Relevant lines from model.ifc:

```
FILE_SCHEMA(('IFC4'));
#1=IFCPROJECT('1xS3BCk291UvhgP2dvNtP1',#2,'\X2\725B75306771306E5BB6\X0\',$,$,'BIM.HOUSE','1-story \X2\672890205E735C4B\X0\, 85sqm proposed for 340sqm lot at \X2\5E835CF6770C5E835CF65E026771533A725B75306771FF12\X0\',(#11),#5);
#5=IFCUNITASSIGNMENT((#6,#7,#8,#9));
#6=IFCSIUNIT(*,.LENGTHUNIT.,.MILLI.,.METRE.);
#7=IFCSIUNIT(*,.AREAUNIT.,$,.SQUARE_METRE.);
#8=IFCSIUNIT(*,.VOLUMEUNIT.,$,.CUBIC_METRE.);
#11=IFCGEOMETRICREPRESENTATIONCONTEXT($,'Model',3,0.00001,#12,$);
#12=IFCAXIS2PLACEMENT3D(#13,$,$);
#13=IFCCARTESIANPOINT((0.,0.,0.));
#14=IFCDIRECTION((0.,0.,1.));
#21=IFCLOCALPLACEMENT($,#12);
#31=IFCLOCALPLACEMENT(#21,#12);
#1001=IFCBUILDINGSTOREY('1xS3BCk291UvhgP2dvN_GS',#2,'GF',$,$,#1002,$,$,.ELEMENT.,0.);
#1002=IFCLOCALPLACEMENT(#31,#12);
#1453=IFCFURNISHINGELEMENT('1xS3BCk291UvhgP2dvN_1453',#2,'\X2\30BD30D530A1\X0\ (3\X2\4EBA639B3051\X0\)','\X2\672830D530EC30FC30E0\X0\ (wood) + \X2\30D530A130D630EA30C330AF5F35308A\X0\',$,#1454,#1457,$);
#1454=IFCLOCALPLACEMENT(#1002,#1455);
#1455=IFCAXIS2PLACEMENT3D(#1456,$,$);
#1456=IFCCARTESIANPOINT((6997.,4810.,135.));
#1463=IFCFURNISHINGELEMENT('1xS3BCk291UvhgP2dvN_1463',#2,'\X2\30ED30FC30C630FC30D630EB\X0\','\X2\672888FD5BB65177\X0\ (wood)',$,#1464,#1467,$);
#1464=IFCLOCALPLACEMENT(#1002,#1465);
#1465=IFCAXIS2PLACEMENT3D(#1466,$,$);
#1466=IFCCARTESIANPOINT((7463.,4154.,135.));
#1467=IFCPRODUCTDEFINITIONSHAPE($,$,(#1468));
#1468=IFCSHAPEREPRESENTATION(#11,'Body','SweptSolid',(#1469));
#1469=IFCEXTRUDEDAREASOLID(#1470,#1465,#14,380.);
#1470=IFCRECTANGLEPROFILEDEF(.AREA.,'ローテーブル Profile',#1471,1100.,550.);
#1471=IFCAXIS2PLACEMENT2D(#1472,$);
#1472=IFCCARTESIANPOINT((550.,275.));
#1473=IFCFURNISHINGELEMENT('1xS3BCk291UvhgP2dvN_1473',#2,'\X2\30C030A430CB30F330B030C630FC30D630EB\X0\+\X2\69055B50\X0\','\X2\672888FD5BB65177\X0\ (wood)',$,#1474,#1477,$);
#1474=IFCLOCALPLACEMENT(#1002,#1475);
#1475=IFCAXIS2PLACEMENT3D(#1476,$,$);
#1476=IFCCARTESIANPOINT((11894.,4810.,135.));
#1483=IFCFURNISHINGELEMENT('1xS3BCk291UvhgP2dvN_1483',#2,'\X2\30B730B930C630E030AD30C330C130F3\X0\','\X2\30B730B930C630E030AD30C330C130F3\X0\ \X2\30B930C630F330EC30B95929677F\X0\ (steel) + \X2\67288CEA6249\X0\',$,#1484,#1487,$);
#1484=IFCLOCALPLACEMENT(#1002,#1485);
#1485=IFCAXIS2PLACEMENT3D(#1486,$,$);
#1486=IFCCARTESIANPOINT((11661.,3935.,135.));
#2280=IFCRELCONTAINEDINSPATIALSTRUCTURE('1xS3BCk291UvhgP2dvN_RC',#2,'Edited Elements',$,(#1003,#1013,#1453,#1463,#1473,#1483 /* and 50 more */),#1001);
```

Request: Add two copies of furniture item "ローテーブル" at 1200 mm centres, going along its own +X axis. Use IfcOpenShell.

```python
import ifcopenshell
import ifcopenshell.api.geometry
import ifcopenshell.api.root
import ifcopenshell.util.element
import ifcopenshell.util.placement

model = ifcopenshell.open("model.ifc")


def reuse_history(source, copy):
    """copy_class also copies each property set's owner history, people and application; keep the originals."""
    for rel in copy.IsDefinedBy:
        if rel.is_a("IfcRelDefinesByProperties") and (history := rel.RelatingPropertyDefinition.OwnerHistory):
            rel.RelatingPropertyDefinition.OwnerHistory = source.OwnerHistory
            ifcopenshell.util.element.remove_deep2(model, history)


source = model.by_guid("1xS3BCk291UvhgP2dvN_1463")
base = ifcopenshell.util.placement.get_local_placement(source.ObjectPlacement)
step = base[:3, 0] * 1200.0

for i in range(1, 3):
    copy = ifcopenshell.api.root.copy_class(model, product=source)
    copy.Representation = ifcopenshell.util.element.copy_deep(
        model, source.Representation, exclude=["IfcGeometricRepresentationContext", "IfcRepresentationMap"]
    )
    reuse_history(source, copy)
    matrix = base.copy()
    matrix[:3, 3] += i * step
    print("added at", matrix[:3, 3].round(3) + 0.0)
    ifcopenshell.api.geometry.edit_object_placement(model, product=copy, matrix=matrix, is_si=False)

model.write("model_rev.ifc")
```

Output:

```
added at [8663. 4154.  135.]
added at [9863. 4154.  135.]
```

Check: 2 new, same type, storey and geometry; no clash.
